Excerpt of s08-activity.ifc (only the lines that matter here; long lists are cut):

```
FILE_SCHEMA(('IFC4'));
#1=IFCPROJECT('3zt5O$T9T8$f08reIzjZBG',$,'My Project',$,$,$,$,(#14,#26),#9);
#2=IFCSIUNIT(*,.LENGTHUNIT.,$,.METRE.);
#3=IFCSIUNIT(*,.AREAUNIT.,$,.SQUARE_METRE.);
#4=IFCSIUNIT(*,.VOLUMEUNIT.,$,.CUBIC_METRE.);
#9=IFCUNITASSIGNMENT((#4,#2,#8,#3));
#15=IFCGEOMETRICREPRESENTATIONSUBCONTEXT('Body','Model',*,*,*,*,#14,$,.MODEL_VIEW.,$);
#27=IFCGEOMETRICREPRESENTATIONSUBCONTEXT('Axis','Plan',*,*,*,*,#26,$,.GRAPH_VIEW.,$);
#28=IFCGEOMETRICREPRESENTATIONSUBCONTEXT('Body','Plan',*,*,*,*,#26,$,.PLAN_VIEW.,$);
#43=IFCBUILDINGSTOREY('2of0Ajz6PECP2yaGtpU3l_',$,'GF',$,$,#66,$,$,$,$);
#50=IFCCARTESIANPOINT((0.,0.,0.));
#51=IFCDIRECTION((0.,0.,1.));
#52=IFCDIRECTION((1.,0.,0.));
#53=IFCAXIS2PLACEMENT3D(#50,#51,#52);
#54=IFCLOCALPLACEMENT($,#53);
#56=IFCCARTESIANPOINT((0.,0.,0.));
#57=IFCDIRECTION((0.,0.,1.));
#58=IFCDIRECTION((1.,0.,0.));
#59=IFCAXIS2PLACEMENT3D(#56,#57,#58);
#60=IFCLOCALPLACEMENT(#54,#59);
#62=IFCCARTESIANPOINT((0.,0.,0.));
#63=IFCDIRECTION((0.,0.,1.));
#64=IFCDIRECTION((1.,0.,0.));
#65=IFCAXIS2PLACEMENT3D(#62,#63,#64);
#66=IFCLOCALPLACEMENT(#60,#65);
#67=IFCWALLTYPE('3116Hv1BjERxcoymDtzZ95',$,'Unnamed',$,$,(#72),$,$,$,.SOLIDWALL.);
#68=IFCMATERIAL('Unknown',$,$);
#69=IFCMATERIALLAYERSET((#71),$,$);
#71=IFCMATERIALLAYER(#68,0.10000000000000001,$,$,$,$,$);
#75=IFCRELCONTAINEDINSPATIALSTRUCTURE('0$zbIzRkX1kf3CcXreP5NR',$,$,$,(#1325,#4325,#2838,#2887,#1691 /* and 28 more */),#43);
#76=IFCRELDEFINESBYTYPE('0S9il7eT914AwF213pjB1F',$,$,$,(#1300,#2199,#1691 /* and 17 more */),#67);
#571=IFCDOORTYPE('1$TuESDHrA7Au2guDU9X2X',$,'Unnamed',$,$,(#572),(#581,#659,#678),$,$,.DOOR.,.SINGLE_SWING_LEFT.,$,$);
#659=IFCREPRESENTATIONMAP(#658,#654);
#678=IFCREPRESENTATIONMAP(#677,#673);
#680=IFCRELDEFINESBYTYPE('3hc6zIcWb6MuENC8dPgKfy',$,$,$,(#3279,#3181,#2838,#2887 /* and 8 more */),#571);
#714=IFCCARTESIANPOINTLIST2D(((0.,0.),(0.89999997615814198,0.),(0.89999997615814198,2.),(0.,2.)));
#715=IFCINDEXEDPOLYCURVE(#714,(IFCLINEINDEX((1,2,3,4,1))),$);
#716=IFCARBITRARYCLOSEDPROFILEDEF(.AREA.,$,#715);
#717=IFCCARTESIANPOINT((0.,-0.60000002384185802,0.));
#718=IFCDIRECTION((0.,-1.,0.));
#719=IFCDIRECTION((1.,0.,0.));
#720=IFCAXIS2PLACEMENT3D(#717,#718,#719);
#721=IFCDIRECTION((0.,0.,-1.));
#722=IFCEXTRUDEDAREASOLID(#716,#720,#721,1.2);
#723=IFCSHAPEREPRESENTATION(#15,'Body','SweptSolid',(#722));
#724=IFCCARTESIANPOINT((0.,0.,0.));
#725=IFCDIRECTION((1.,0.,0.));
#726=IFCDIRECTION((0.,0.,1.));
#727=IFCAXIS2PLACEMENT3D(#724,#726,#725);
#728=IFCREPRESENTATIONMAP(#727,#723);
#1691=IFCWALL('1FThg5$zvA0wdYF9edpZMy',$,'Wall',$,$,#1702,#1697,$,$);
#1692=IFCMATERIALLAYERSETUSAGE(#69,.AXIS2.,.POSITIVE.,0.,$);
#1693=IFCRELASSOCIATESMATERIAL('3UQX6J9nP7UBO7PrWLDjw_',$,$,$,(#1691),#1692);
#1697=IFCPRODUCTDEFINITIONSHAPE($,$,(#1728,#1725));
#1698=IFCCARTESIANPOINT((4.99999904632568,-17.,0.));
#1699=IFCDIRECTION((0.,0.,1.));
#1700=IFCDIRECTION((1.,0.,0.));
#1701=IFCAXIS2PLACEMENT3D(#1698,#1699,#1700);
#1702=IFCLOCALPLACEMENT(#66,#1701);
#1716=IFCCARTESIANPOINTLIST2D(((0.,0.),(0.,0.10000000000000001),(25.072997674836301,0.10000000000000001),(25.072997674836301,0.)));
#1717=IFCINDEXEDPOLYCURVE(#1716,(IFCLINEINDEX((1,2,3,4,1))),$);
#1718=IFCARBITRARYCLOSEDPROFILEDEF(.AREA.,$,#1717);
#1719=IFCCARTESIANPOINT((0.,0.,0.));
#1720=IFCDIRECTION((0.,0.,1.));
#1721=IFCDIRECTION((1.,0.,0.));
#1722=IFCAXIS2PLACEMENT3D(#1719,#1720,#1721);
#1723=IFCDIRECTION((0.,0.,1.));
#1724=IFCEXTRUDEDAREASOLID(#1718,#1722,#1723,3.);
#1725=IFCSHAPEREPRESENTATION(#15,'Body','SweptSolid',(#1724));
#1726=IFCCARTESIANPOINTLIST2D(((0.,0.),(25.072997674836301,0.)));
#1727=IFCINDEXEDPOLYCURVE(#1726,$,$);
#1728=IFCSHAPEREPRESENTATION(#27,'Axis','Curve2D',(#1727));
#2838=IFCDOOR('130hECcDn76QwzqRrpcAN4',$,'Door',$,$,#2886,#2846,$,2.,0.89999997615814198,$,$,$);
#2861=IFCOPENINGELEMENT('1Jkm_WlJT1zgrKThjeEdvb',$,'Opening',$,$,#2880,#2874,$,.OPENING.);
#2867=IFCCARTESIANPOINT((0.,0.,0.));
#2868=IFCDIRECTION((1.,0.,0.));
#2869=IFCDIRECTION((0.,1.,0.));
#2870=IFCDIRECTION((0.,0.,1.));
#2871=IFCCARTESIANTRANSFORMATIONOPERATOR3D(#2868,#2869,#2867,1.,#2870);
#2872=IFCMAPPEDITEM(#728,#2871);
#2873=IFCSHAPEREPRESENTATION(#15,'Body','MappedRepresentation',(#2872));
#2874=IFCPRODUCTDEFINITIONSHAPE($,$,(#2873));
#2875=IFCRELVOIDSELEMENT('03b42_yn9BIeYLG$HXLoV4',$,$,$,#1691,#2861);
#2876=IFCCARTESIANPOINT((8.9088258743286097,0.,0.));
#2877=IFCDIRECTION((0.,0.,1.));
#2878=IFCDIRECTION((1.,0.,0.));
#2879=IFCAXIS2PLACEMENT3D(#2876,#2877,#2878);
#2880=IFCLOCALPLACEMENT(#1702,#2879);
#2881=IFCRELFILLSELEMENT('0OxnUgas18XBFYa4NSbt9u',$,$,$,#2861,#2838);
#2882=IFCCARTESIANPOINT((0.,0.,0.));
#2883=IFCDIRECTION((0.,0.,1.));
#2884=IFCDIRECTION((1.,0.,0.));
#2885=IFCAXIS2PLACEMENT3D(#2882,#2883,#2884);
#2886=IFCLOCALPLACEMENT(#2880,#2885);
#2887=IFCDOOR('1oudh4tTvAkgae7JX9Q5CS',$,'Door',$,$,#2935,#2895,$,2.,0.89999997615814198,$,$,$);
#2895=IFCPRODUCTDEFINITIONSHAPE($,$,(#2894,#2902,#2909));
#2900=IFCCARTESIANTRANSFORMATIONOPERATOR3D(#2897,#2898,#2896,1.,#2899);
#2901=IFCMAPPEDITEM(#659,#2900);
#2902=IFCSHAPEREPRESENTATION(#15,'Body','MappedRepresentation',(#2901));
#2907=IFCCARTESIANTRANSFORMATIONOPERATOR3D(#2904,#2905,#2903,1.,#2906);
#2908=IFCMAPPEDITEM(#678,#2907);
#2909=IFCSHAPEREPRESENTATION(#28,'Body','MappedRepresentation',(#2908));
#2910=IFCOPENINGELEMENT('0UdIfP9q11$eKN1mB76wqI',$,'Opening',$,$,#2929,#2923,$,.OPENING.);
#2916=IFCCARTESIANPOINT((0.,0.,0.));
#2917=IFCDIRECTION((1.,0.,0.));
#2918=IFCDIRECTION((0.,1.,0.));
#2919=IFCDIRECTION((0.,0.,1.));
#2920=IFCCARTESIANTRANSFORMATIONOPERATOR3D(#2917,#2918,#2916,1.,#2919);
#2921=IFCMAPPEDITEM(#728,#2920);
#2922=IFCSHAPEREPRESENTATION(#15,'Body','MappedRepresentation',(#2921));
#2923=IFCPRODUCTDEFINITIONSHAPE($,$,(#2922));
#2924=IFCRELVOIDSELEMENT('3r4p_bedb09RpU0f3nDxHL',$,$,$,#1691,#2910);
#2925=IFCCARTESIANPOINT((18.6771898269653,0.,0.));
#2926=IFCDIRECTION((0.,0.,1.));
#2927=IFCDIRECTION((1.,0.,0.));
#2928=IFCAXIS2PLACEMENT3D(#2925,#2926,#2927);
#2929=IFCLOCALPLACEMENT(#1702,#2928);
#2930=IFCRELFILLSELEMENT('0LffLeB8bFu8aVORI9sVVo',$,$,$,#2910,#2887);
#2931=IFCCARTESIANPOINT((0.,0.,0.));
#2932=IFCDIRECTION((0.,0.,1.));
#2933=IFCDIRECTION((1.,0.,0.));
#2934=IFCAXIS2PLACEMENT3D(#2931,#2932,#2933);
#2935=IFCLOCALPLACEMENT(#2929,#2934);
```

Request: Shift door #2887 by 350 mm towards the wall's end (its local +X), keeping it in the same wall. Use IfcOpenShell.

```python
import ifcopenshell
import ifcopenshell.api.geometry
import ifcopenshell.util.placement

model = ifcopenshell.open("s08-activity.ifc")

door = model.by_guid("1oudh4tTvAkgae7JX9Q5CS")
opening = door.FillsVoids[0].RelatingOpeningElement
wall = opening.VoidsElements[0].RelatingBuildingElement

wall_matrix = ifcopenshell.util.placement.get_local_placement(wall.ObjectPlacement)
shift = wall_matrix[:3, 0] * 0.35
before = ifcopenshell.util.placement.get_local_placement(door.ObjectPlacement)[:3, 3].copy()

# The door is placed relative to its opening, so it follows when the opening moves.
matrix = ifcopenshell.util.placement.get_local_placement(opening.ObjectPlacement)
matrix[:3, 3] += shift
ifcopenshell.api.geometry.edit_object_placement(
    model, product=opening, matrix=matrix, is_si=False, should_transform_children=True
)

after = ifcopenshell.util.placement.get_local_placement(door.ObjectPlacement)[:3, 3]
print("door moved by", (after - before).round(3) + 0.0)

model.write("s08-activity_rev.ifc")
```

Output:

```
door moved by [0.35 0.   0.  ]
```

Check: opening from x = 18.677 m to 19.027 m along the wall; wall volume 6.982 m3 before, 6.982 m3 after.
